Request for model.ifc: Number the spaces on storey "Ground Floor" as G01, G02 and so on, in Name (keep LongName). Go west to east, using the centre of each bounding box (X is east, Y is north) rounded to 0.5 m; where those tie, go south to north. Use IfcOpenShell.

First a look at what the model holds.

```python
import ifcopenshell
import ifcopenshell.util.element
import ifcopenshell.util.placement

model = ifcopenshell.open("model.ifc")
print(model.schema)
storey = next(s for s in model.by_type("IfcBuildingStorey") if s.Name == "Ground Floor")
spaces = [e for e in ifcopenshell.util.element.get_decomposition(storey) if e.is_a("IfcSpace")]
for e in sorted(spaces, key=lambda e: e.id()):
    origin = ifcopenshell.util.placement.get_local_placement(e.ObjectPlacement)[:3, 3]
    print(e.id(), e.Name, e.LongName, origin.round(2) + 0.0, sep=" | ")
```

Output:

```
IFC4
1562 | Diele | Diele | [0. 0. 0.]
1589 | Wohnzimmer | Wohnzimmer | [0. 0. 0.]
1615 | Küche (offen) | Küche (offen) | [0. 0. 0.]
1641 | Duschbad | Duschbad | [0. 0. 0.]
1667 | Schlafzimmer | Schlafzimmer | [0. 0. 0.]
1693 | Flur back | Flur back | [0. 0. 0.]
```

```python
import ifcopenshell
import ifcopenshell.geom
import ifcopenshell.util.element
import ifcopenshell.util.shape

model = ifcopenshell.open("model.ifc")
settings = ifcopenshell.geom.settings()
settings.set("use-world-coords", True)


def centre(element):
    shape = ifcopenshell.geom.create_shape(settings, element)
    return ifcopenshell.util.shape.get_bbox_centroid(shape.geometry)


storey = next(s for s in model.by_type("IfcBuildingStorey") if s.Name == "Ground Floor")
spaces = [e for e in ifcopenshell.util.element.get_decomposition(storey) if e.is_a("IfcSpace")]

# Insertion points can sit at a corner or the storey origin, so sort by the geometry (in metres).
centres = {e: centre(e) for e in spaces}
spaces.sort(key=lambda e: (round(centres[e][0] / 0.5), centres[e][1]))

for i, e in enumerate(spaces, start=1):
    number = f"G{i:02d}"
    e.Name = number
    print(e.id(), number)

model.write("model_v2.ifc")
```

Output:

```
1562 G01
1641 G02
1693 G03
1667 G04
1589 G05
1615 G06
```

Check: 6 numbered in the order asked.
